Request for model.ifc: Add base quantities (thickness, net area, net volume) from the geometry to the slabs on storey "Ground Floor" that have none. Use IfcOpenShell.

First a look at what the model holds.

```python
import ifcopenshell
import ifcopenshell.util.element
import ifcopenshell.util.unit

model = ifcopenshell.open("model.ifc")
print(model.schema)
for unit_type in ("LENGTHUNIT", "AREAUNIT", "VOLUMEUNIT"):
    print(unit_type, ifcopenshell.util.unit.calculate_unit_scale(model, unit_type))
storey = next(s for s in model.by_type("IfcBuildingStorey") if s.Name == "Ground Floor")
slabs = [e for e in ifcopenshell.util.element.get_decomposition(storey) if e.is_a("IfcSlab")]
for e in sorted(slabs, key=lambda e: e.id()):
    print(e.id(), e.is_a(), e.Name, list(ifcopenshell.util.element.get_psets(e, qtos_only=True)), sep=" | ")
```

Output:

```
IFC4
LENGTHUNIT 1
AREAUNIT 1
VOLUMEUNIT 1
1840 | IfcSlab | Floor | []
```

```python
import ifcopenshell
import ifcopenshell.api.pset
import ifcopenshell.geom
import ifcopenshell.util.element
import ifcopenshell.util.shape
import ifcopenshell.util.unit

model = ifcopenshell.open("model.ifc")
unit_scale = ifcopenshell.util.unit.calculate_unit_scale(model)
area_scale = ifcopenshell.util.unit.calculate_unit_scale(model, "AREAUNIT")
volume_scale = ifcopenshell.util.unit.calculate_unit_scale(model, "VOLUMEUNIT")
settings = ifcopenshell.geom.settings()

storey = next(s for s in model.by_type("IfcBuildingStorey") if s.Name == "Ground Floor")
slabs = [e for e in ifcopenshell.util.element.get_decomposition(storey) if e.is_a("IfcSlab")]

for e in sorted(slabs, key=lambda e: e.id()):
    if ifcopenshell.util.element.get_psets(e, qtos_only=True, should_inherit=False):
        continue
    # Geometry comes back in metres, in the element's own axes.
    shape = ifcopenshell.geom.create_shape(settings, e)
    values = {
        "Width": ifcopenshell.util.shape.get_z(shape.geometry) / unit_scale,
        "NetArea": ifcopenshell.util.shape.get_footprint_area(shape.geometry) / area_scale,
        "NetVolume": ifcopenshell.util.shape.get_volume(shape.geometry) / volume_scale,
    }
    qto = ifcopenshell.api.pset.add_qto(model, product=e, name="Qto_SlabBaseQuantities")
    ifcopenshell.api.pset.edit_qto(model, qto=qto, properties=values)
    print(e.id(), {k: round(v, 3) for k, v in values.items()})

model.write("model_updated.ifc")
```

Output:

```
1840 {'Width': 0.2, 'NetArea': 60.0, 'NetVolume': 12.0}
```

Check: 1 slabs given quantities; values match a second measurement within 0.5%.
